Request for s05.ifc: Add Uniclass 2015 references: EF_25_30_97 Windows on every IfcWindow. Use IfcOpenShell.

First a look at what the model holds.

```python
import ifcopenshell

model = ifcopenshell.open("s05.ifc")
print(model.schema)
print("classifications:", [c.Name for c in model.by_type("IfcClassification")])
for ifc_class in ("IfcDoor", "IfcRoof", "IfcStair", "IfcWall", "IfcWindow"):
    print(ifc_class, len(model.by_type(ifc_class)))
```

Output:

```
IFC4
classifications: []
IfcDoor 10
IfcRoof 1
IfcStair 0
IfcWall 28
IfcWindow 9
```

```python
import ifcopenshell
import ifcopenshell.api.classification

model = ifcopenshell.open("s05.ifc")

system = ifcopenshell.api.classification.add_classification(model, classification="Uniclass 2015")

codes = {
    "IfcWindow": ("EF_25_30_97", "Windows"),
}
for ifc_class, (code, name) in codes.items():
    products = model.by_type(ifc_class)
    ifcopenshell.api.classification.add_reference(
        model, products=products, classification=system, identification=code, name=name
    )
    print(code, len(products))

model.write("s05_updated.ifc")
```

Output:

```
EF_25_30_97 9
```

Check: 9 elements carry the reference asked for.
